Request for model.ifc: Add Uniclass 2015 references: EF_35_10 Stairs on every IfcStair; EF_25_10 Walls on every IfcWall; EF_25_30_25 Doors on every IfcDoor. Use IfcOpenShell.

First a look at what the model holds.

```python
import ifcopenshell

model = ifcopenshell.open("model.ifc")
print(model.schema)
print("classifications:", [c.Name for c in model.by_type("IfcClassification")])
for ifc_class in ("IfcDoor", "IfcRoof", "IfcStair", "IfcWall", "IfcWindow"):
    print(ifc_class, len(model.by_type(ifc_class)))
```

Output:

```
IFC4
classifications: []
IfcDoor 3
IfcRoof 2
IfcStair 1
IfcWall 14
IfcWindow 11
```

```python
import ifcopenshell
import ifcopenshell.api.classification

model = ifcopenshell.open("model.ifc")

system = ifcopenshell.api.classification.add_classification(model, classification="Uniclass 2015")

codes = {
    "IfcStair": ("EF_35_10", "Stairs"),
    "IfcWall": ("EF_25_10", "Walls"),
    "IfcDoor": ("EF_25_30_25", "Doors"),
}
for ifc_class, (code, name) in codes.items():
    products = model.by_type(ifc_class)
    ifcopenshell.api.classification.add_reference(
        model, products=products, classification=system, identification=code, name=name
    )
    print(code, len(products))

model.write("model-out.ifc")
```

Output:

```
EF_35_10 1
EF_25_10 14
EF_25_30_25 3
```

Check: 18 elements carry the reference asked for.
